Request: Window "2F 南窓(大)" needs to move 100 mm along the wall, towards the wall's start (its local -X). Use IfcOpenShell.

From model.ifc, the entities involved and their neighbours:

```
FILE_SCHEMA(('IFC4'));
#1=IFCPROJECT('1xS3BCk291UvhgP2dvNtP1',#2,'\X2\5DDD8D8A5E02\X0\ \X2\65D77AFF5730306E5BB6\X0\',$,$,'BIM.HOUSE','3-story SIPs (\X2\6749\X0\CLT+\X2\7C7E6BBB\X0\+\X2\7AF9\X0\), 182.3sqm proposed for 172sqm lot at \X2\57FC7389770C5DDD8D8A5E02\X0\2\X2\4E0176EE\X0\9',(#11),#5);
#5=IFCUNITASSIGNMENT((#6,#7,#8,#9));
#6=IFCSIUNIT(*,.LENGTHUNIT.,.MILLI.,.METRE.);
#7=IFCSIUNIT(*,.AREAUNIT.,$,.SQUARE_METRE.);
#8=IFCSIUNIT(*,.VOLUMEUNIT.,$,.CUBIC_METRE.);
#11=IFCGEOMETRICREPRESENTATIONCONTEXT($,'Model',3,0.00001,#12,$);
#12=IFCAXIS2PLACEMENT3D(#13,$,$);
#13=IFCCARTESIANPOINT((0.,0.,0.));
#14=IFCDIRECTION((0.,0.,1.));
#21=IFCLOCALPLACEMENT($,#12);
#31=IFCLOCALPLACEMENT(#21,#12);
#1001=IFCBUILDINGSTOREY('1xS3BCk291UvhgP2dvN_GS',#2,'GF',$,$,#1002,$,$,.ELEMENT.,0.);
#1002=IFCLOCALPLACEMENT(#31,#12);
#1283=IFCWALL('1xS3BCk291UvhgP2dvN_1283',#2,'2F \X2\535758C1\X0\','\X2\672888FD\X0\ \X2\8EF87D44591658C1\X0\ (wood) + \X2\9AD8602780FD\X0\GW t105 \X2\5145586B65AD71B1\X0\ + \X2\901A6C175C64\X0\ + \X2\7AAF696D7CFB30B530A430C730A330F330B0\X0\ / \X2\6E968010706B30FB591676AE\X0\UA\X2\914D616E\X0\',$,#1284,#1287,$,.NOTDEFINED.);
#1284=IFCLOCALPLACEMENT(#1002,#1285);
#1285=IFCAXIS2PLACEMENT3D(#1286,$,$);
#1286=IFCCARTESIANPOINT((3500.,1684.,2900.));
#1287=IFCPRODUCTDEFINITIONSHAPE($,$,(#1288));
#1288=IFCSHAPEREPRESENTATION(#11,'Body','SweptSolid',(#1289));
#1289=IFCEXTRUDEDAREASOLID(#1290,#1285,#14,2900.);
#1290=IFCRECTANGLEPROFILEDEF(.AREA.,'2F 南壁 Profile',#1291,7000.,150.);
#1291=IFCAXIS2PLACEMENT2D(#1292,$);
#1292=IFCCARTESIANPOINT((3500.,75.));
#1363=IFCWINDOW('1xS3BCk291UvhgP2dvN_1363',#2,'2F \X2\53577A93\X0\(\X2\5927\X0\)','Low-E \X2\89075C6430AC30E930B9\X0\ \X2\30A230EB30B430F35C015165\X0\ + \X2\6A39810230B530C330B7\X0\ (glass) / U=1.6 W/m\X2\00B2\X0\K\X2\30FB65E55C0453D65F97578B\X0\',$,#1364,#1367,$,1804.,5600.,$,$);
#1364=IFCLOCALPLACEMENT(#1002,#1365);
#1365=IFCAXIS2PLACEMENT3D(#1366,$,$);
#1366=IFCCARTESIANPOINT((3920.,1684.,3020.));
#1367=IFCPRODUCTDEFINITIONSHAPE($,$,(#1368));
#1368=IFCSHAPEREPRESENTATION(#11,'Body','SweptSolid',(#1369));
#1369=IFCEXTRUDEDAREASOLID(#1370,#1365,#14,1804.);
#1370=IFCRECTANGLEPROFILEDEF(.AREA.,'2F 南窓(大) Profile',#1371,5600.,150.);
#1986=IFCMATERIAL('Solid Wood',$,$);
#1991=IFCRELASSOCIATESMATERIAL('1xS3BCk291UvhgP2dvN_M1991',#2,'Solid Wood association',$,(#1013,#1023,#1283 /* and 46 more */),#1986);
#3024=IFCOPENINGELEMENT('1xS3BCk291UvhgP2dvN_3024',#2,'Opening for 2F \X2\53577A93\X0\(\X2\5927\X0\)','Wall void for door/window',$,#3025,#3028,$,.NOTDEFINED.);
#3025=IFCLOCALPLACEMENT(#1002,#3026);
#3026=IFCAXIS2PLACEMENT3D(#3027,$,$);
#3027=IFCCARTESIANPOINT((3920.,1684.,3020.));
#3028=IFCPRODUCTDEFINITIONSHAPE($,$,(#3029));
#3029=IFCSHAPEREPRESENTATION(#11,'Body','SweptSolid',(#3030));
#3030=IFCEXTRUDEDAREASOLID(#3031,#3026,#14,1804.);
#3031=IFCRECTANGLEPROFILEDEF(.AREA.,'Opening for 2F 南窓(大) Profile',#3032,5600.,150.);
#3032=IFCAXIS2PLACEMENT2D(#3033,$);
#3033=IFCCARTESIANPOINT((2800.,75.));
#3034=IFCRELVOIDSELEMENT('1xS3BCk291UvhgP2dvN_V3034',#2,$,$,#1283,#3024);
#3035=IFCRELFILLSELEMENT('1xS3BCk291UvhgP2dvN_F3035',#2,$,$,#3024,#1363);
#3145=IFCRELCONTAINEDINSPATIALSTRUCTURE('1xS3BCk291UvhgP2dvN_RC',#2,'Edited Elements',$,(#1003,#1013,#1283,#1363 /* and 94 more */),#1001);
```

```python
import ifcopenshell
import ifcopenshell.api.geometry
import ifcopenshell.util.placement
import ifcopenshell.util.unit

model = ifcopenshell.open("model.ifc")
unit_scale = ifcopenshell.util.unit.calculate_unit_scale(model)

window = model.by_guid("1xS3BCk291UvhgP2dvN_1363")
opening = window.FillsVoids[0].RelatingOpeningElement
wall = opening.VoidsElements[0].RelatingBuildingElement

wall_matrix = ifcopenshell.util.placement.get_local_placement(wall.ObjectPlacement)
shift = wall_matrix[:3, 0] * -0.1 / unit_scale
before = ifcopenshell.util.placement.get_local_placement(window.ObjectPlacement)[:3, 3].copy()

# The window is not placed relative to its opening, so move both.
for product in (opening, window):
    matrix = ifcopenshell.util.placement.get_local_placement(product.ObjectPlacement)
    matrix[:3, 3] += shift
    ifcopenshell.api.geometry.edit_object_placement(model, product=product, matrix=matrix, is_si=False)

after = ifcopenshell.util.placement.get_local_placement(window.ObjectPlacement)[:3, 3]
print("window moved by", (after - before).round(3) + 0.0)

model.write("model_v2.ifc")
```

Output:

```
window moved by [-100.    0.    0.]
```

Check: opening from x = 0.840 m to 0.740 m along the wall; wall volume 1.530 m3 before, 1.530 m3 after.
